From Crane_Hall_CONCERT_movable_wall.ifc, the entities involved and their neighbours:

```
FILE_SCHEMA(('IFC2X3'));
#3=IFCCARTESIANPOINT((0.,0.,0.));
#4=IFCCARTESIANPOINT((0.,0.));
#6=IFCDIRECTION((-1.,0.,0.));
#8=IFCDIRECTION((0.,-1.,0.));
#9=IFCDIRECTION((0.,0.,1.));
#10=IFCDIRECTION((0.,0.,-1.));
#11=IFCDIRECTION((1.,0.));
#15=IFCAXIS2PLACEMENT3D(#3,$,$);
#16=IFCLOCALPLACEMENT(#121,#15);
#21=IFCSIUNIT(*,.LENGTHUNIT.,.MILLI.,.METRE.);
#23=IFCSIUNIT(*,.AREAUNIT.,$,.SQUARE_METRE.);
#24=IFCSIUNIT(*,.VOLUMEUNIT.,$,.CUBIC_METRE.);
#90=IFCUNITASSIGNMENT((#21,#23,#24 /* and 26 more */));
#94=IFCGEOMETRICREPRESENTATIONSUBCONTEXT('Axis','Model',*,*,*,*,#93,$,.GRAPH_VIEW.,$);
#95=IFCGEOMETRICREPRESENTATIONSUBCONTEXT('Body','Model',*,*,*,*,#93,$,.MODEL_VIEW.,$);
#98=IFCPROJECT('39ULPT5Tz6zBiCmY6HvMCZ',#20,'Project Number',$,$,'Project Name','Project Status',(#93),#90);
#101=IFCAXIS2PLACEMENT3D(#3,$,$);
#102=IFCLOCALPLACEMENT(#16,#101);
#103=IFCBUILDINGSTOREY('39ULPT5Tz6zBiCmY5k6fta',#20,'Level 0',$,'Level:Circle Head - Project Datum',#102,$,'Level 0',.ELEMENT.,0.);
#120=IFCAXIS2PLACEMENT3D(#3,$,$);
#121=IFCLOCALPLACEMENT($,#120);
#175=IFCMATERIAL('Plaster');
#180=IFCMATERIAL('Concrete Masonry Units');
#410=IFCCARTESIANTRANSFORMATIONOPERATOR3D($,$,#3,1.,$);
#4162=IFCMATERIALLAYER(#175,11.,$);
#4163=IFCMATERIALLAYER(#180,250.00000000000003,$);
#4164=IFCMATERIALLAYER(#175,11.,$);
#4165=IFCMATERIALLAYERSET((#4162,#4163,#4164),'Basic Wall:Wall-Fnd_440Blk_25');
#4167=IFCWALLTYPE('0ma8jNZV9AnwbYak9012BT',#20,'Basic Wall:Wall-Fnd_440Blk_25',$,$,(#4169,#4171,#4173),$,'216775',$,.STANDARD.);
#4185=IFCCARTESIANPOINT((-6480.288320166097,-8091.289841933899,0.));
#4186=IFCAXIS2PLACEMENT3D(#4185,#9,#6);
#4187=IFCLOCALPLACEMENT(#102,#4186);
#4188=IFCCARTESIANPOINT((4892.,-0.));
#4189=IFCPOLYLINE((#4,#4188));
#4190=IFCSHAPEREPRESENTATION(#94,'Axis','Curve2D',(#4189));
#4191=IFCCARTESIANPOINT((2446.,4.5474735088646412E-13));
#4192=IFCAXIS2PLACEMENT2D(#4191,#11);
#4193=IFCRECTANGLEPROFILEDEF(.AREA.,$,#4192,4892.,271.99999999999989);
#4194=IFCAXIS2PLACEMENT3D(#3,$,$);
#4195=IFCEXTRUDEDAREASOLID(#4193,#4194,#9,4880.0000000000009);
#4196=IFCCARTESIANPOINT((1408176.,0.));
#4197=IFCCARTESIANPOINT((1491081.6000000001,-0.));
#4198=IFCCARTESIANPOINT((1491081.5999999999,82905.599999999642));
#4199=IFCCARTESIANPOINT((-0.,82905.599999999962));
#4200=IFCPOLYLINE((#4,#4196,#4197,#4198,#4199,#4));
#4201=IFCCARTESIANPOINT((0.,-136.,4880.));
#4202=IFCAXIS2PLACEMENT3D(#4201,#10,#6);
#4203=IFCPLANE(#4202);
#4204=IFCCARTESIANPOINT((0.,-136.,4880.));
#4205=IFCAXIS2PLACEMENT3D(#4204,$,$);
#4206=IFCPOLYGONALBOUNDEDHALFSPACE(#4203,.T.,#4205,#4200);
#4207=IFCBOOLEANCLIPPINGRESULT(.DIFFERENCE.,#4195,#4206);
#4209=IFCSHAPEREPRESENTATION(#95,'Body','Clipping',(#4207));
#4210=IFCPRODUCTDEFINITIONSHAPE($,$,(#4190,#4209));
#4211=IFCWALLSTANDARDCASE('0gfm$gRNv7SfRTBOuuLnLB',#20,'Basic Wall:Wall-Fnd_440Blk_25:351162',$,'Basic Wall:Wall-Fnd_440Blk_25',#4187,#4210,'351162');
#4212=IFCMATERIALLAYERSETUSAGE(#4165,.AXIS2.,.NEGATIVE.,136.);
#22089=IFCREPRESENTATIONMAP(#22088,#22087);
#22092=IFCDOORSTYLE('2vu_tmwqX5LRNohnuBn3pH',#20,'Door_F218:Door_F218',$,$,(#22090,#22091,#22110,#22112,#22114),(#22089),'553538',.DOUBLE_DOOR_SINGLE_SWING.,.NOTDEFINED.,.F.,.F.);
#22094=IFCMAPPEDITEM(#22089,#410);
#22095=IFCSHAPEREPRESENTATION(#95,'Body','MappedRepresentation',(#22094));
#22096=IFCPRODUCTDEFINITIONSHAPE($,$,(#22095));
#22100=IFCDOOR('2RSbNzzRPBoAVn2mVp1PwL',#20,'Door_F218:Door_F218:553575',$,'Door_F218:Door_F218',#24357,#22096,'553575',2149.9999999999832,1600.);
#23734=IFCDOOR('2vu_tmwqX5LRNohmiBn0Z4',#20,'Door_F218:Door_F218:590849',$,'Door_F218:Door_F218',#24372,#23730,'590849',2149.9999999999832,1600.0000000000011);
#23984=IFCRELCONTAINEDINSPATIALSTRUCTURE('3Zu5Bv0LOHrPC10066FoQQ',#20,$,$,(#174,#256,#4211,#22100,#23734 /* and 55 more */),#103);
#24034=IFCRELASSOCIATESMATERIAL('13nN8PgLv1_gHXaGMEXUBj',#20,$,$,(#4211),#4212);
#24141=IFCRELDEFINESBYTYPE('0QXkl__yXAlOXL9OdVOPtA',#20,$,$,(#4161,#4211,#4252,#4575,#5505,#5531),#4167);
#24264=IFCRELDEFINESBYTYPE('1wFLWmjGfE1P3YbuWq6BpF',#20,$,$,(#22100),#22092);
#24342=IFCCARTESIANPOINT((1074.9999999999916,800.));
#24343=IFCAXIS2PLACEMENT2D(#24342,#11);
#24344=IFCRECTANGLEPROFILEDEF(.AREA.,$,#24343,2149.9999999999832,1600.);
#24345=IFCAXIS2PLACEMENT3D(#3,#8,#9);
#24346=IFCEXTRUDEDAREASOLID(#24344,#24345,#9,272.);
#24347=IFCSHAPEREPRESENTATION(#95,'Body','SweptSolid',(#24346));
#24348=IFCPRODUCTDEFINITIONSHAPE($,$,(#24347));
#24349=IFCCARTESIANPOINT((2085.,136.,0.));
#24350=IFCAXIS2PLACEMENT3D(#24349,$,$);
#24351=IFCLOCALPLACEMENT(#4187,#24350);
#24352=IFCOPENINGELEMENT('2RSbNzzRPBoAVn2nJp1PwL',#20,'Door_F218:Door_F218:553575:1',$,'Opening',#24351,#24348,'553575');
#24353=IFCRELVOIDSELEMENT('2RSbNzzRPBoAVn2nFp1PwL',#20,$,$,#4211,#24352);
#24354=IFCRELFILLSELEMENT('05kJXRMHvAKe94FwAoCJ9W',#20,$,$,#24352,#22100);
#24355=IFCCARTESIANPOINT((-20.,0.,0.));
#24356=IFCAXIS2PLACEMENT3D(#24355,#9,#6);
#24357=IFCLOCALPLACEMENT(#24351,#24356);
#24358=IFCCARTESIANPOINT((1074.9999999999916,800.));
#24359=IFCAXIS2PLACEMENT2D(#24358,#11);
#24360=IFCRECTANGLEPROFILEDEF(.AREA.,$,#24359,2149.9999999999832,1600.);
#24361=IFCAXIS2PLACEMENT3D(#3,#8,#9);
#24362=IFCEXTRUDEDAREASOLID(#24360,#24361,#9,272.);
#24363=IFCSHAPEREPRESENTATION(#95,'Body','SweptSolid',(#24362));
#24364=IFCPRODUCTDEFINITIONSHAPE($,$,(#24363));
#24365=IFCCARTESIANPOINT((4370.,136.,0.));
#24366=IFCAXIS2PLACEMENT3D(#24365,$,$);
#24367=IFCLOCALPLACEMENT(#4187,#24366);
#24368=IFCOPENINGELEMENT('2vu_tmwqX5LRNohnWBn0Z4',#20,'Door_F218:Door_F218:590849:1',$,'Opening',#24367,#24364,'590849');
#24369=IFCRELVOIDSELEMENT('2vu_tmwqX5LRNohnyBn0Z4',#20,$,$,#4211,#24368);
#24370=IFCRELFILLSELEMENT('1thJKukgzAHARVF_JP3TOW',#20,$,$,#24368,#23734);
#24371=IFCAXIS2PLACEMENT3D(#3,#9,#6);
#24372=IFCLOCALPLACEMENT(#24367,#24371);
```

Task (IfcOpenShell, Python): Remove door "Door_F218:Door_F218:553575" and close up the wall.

```python
import ifcopenshell
import ifcopenshell.api.feature
import ifcopenshell.api.root
import ifcopenshell.geom
import ifcopenshell.util.shape

model = ifcopenshell.open("Crane_Hall_CONCERT_movable_wall.ifc")
settings = ifcopenshell.geom.settings()


def volume(element):
    """Net volume in cubic metres, openings subtracted."""
    shape = ifcopenshell.geom.create_shape(settings, element)
    return ifcopenshell.util.shape.get_volume(shape.geometry)


door = model.by_guid("2RSbNzzRPBoAVn2mVp1PwL")
opening = door.FillsVoids[0].RelatingOpeningElement
wall = opening.VoidsElements[0].RelatingBuildingElement
before = volume(wall)

ifcopenshell.api.root.remove_product(model, product=door)
ifcopenshell.api.feature.remove_feature(model, feature=opening)

after = volume(wall)

print(f"wall volume {before:.3f} -> {after:.3f} m3")

model.write("Crane_Hall_CONCERT_movable_wall_updated.ifc")
```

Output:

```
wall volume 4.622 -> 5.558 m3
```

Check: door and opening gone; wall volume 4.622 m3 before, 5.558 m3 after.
